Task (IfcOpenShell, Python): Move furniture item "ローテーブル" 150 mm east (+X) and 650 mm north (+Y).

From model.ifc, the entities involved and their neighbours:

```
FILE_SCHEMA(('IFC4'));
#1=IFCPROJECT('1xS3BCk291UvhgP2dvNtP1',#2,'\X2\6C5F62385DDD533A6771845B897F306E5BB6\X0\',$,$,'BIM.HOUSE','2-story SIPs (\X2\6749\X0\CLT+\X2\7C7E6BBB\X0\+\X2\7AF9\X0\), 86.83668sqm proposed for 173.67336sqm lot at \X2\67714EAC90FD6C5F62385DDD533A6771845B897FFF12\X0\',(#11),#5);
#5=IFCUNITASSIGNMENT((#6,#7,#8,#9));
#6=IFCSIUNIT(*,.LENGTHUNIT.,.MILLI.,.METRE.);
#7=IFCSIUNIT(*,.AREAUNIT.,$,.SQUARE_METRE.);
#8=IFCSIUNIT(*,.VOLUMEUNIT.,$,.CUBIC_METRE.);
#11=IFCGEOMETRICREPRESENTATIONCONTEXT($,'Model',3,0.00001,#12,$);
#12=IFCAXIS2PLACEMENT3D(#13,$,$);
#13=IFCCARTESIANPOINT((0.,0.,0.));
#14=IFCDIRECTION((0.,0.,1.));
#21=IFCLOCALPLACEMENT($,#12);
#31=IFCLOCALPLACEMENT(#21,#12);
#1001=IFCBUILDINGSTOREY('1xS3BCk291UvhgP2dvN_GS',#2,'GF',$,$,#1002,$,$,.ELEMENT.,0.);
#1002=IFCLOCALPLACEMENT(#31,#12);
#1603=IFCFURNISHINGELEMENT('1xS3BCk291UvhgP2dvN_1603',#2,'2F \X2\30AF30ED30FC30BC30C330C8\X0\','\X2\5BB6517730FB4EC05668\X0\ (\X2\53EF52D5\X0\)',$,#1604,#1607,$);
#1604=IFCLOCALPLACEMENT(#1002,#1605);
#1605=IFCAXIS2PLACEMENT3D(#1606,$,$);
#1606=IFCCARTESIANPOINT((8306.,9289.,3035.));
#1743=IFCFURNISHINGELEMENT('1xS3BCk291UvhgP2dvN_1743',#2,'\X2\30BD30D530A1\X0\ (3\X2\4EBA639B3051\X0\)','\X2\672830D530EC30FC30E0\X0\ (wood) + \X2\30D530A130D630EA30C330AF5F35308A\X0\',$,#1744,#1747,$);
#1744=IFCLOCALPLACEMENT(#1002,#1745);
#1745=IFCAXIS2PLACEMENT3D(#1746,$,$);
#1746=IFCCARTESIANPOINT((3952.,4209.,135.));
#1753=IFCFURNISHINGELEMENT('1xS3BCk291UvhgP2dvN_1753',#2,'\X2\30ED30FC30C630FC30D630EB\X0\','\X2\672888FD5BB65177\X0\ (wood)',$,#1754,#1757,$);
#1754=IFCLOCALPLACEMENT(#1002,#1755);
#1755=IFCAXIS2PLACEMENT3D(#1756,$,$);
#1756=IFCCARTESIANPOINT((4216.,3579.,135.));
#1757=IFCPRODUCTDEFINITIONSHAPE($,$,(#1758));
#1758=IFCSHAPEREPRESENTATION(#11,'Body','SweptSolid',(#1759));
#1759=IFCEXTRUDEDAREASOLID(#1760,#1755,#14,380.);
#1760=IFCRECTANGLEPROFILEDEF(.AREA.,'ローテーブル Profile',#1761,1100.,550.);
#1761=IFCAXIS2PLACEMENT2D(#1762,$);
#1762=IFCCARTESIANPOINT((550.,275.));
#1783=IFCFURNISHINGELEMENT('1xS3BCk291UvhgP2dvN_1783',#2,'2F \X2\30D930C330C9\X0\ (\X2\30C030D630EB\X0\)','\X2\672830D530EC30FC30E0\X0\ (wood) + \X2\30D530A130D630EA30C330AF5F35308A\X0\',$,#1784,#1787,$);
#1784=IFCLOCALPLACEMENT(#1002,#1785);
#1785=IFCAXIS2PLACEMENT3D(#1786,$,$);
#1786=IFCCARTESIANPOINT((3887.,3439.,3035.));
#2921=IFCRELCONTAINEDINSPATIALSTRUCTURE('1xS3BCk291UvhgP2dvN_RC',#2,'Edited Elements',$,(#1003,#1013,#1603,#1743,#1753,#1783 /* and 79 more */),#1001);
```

```python
import ifcopenshell
import ifcopenshell.api.geometry
import ifcopenshell.util.placement

model = ifcopenshell.open("model.ifc")

item = model.by_id(1753)
matrix = ifcopenshell.util.placement.get_local_placement(item.ObjectPlacement)
matrix[0, 3] += 150.0
matrix[1, 3] += 650.0
ifcopenshell.api.geometry.edit_object_placement(model, product=item, matrix=matrix, is_si=False)

print(ifcopenshell.util.placement.get_local_placement(item.ObjectPlacement).round(3) + 0.0)

model.write("model_rev.ifc")
```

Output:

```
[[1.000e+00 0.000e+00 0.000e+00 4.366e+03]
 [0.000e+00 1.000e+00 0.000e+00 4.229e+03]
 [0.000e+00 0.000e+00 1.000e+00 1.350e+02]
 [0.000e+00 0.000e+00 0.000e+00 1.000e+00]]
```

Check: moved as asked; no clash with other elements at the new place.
